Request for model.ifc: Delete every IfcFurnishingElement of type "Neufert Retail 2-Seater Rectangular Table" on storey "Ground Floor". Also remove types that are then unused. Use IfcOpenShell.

First a look at what the model holds.

```python
import ifcopenshell
import ifcopenshell.util.element

model = ifcopenshell.open("model.ifc")
print(model.schema)
storey = next(s for s in model.by_type("IfcBuildingStorey") if s.Name == "Ground Floor")
furniture = [e for e in ifcopenshell.util.element.get_decomposition(storey) if e.is_a("IfcFurnishingElement")]
seen = {}
for e in furniture:
    element_type = ifcopenshell.util.element.get_type(e)
    name = element_type.Name if element_type not in (None, e) else None
    seen[name] = seen.get(name, 0) + 1
for name, count in sorted(seen.items(), key=str):
    print(count, "x", name)
```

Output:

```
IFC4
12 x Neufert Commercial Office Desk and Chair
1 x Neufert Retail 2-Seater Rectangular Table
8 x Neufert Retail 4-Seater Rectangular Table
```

```python
import ifcopenshell
import ifcopenshell.api.root
import ifcopenshell.util.element

model = ifcopenshell.open("model.ifc")

storey = next(s for s in model.by_type("IfcBuildingStorey") if s.Name == "Ground Floor")
furniture = [e for e in ifcopenshell.util.element.get_decomposition(storey) if e.is_a("IfcFurnishingElement")]
targets = [e for e in furniture if (t := ifcopenshell.util.element.get_type(e)) not in (None, e) and t.Name == "Neufert Retail 2-Seater Rectangular Table"]
types = {ifcopenshell.util.element.get_type(e) for e in targets} - {None, *targets}

for e in targets:
    ifcopenshell.api.root.remove_product(model, product=e)
print(len(targets), "removed")

unused = [t for t in types if not ifcopenshell.util.element.get_types(t)]
for t in unused:
    ifcopenshell.api.root.remove_product(model, product=t)
print(len(unused), "unused types removed")

model.write("model_edited.ifc")
```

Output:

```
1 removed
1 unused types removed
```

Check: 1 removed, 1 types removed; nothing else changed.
